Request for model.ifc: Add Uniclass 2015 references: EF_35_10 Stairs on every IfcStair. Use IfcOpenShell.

First a look at what the model holds.

```python
import ifcopenshell

model = ifcopenshell.open("model.ifc")
print(model.schema)
print("classifications:", [c.Name for c in model.by_type("IfcClassification")])
for ifc_class in ("IfcDoor", "IfcRoof", "IfcStair", "IfcWall", "IfcWindow"):
    print(ifc_class, len(model.by_type(ifc_class)))
```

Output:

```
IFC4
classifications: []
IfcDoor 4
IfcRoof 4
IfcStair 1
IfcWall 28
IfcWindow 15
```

```python
import ifcopenshell
import ifcopenshell.api.classification

model = ifcopenshell.open("model.ifc")

system = ifcopenshell.api.classification.add_classification(model, classification="Uniclass 2015")

codes = {
    "IfcStair": ("EF_35_10", "Stairs"),
}
for ifc_class, (code, name) in codes.items():
    products = model.by_type(ifc_class)
    ifcopenshell.api.classification.add_reference(
        model, products=products, classification=system, identification=code, name=name
    )
    print(code, len(products))

model.write("model_edited.ifc")
```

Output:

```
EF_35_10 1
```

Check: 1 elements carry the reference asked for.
